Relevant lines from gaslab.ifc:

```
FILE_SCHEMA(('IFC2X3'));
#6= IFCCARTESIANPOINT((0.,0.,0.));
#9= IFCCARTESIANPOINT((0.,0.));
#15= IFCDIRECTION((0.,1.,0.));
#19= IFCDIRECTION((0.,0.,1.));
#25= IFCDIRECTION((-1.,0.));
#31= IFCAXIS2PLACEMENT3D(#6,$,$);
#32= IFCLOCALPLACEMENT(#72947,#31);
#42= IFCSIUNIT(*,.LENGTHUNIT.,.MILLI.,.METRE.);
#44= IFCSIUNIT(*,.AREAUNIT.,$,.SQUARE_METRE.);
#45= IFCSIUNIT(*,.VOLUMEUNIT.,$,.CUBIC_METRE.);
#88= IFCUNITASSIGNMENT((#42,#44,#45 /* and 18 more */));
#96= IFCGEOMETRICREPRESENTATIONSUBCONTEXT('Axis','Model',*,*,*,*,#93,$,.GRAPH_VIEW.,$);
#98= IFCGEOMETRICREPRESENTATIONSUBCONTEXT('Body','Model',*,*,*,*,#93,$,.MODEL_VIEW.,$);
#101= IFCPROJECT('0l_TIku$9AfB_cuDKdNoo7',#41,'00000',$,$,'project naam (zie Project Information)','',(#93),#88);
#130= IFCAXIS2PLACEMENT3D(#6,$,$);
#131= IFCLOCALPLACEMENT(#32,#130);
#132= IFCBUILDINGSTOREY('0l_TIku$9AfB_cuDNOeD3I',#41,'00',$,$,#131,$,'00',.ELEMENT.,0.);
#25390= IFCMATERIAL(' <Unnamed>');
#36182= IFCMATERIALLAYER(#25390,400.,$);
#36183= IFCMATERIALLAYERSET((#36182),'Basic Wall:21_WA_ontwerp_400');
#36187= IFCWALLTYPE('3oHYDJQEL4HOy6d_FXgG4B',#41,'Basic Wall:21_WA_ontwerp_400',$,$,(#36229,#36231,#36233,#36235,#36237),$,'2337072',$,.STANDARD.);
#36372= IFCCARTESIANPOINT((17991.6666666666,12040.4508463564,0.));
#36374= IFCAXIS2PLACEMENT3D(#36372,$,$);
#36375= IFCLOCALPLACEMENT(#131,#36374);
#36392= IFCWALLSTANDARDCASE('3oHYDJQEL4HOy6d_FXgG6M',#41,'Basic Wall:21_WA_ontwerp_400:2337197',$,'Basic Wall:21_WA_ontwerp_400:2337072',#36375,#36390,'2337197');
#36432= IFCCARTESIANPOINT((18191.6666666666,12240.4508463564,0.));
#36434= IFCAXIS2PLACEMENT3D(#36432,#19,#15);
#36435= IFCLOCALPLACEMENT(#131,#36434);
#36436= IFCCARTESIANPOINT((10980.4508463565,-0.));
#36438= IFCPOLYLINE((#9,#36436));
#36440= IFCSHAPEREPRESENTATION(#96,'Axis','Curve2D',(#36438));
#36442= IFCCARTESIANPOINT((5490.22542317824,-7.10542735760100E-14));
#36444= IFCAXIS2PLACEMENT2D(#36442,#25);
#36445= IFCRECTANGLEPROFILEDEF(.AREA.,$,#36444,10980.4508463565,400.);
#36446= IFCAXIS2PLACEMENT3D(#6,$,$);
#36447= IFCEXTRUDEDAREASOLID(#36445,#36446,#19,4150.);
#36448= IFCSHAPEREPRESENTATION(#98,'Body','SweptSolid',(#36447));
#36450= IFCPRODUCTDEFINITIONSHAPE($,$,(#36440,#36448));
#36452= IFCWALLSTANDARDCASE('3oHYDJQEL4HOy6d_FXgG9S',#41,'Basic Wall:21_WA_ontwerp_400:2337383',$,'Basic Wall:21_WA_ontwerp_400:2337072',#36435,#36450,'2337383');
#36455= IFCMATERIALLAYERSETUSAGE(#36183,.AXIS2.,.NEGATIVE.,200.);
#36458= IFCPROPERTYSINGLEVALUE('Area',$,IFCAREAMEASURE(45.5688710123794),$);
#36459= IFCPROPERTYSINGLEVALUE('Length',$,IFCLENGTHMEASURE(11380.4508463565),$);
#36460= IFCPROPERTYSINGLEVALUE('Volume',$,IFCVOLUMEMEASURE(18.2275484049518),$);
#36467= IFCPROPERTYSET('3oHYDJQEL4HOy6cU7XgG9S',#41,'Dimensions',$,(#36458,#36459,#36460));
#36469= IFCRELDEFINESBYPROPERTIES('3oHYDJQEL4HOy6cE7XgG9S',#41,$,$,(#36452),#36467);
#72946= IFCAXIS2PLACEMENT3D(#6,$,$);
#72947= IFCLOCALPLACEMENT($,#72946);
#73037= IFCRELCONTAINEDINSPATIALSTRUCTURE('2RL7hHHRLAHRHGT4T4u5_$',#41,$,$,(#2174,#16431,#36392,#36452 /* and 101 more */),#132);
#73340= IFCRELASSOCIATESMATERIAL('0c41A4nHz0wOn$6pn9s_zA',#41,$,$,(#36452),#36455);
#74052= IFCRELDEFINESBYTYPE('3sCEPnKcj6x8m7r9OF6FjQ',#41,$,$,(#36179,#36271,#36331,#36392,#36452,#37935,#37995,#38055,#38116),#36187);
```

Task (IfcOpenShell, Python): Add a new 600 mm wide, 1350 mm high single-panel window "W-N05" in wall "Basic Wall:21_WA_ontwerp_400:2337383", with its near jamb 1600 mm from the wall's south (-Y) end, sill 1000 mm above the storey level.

```python
import numpy as np
import ifcopenshell
import ifcopenshell.api.feature
import ifcopenshell.api.geometry
import ifcopenshell.api.pset
import ifcopenshell.api.root
import ifcopenshell.api.spatial
import ifcopenshell.api.type
import ifcopenshell.geom
import ifcopenshell.util.element
import ifcopenshell.util.placement
import ifcopenshell.util.representation
import ifcopenshell.util.shape
import ifcopenshell.util.unit

model = ifcopenshell.open("gaslab.ifc")
unit_scale = ifcopenshell.util.unit.calculate_unit_scale(model)
area_scale = ifcopenshell.util.unit.calculate_unit_scale(model, "AREAUNIT")
volume_scale = ifcopenshell.util.unit.calculate_unit_scale(model, "VOLUMEUNIT")
settings = ifcopenshell.geom.settings()


def volume(element):
    """Net volume in cubic metres, openings subtracted."""
    shape = ifcopenshell.geom.create_shape(settings, element)
    return ifcopenshell.util.shape.get_volume(shape.geometry)


wall = model.by_id(36452)
storey = ifcopenshell.util.element.get_container(wall, ifc_class="IfcBuildingStorey")
context = ifcopenshell.util.representation.get_context(model, "Model", "Body", "MODEL_VIEW")
before = volume(wall)

width, height, from_end, sill = 0.6, 1.35, 1.6, 1  # metres

# The wall runs along its own X axis, and the end named is its -X end.
wall_shape = ifcopenshell.geom.create_shape(settings, wall)
x, y, z = ifcopenshell.util.shape.get_vertices(wall_shape.geometry).T
start = x.min() + from_end
face, thickness = float(y.min()), float(y.max() - y.min())
wall_matrix = ifcopenshell.util.placement.get_local_placement(wall.ObjectPlacement)
level = ifcopenshell.util.placement.get_local_placement(storey.ObjectPlacement)[2, 3]


def in_wall(x, y):
    """Placement at x, y metres in the wall's axes, at sill height."""
    matrix = wall_matrix.copy()
    matrix[:, 3] = wall_matrix @ np.array([x / unit_scale, y / unit_scale, 0.0, 1.0])
    matrix[2, 3] = level + sill / unit_scale
    return matrix


# Opening: a box that overshoots both wall faces by 50 mm.
opening = ifcopenshell.api.root.create_entity(model, ifc_class="IfcOpeningElement")
box = ifcopenshell.api.geometry.add_wall_representation(
    model, context=context, length=width, height=height, thickness=thickness + 0.1
)
ifcopenshell.api.geometry.assign_representation(model, product=opening, representation=box)
ifcopenshell.api.geometry.edit_object_placement(model, product=opening, matrix=in_wall(start, face - 0.05), is_si=False)
ifcopenshell.api.feature.add_feature(model, feature=opening, element=wall)

window = ifcopenshell.api.root.create_entity(model, ifc_class="IfcWindow", name="W-N05")
window.OverallWidth, window.OverallHeight = width / unit_scale, height / unit_scale
body = ifcopenshell.api.geometry.add_window_representation(
    model,
    context=context,
    overall_width=window.OverallWidth,
    overall_height=window.OverallHeight,
    partition_type="SINGLE_PANEL",
)
ifcopenshell.api.geometry.assign_representation(model, product=window, representation=body)
ifcopenshell.api.spatial.assign_container(model, products=[window], relating_structure=storey)
fills = ifcopenshell.api.feature.add_filling(model, opening=opening, element=window)
fills.OwnerHistory = window.OwnerHistory  # required in IFC2X3

# IFC2X3 keeps the operation on the window style.
style = ifcopenshell.api.root.create_entity(model, ifc_class="IfcWindowStyle", name="W-N05")
style.OperationType, style.ConstructionType = "SINGLE_PANEL", "NOTDEFINED"
style.ParameterTakesPrecedence = style.Sizeable = False
ifcopenshell.api.type.assign_type(model, related_objects=[window], relating_type=style)

# Centre the window in the wall's thickness.
ifcopenshell.api.geometry.edit_object_placement(model, product=window, matrix=in_wall(start, face), is_si=False)
window_shape = ifcopenshell.geom.create_shape(settings, window)
depth = ifcopenshell.util.shape.get_vertices(window_shape.geometry)[:, 1]
offset = face + thickness / 2 - (depth.min() + depth.max()) / 2
ifcopenshell.api.geometry.edit_object_placement(model, product=window, matrix=in_wall(start, offset), is_si=False)

after = volume(wall)

# Update the wall's stored quantities.
pset = model.by_id(ifcopenshell.util.element.get_pset(wall, "Dimensions", should_inherit=False)["id"])
ifcopenshell.api.pset.edit_pset(model, pset=pset, properties={
    "Area": model.create_entity("IfcAreaMeasure", after / thickness / area_scale),
    "Volume": model.create_entity("IfcVolumeMeasure", after / volume_scale),
})

print(f"wall volume {before:.3f} -> {after:.3f} m3")

model.write("gaslab_updated.ifc")
```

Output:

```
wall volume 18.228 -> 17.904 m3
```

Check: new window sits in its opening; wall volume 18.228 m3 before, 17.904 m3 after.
